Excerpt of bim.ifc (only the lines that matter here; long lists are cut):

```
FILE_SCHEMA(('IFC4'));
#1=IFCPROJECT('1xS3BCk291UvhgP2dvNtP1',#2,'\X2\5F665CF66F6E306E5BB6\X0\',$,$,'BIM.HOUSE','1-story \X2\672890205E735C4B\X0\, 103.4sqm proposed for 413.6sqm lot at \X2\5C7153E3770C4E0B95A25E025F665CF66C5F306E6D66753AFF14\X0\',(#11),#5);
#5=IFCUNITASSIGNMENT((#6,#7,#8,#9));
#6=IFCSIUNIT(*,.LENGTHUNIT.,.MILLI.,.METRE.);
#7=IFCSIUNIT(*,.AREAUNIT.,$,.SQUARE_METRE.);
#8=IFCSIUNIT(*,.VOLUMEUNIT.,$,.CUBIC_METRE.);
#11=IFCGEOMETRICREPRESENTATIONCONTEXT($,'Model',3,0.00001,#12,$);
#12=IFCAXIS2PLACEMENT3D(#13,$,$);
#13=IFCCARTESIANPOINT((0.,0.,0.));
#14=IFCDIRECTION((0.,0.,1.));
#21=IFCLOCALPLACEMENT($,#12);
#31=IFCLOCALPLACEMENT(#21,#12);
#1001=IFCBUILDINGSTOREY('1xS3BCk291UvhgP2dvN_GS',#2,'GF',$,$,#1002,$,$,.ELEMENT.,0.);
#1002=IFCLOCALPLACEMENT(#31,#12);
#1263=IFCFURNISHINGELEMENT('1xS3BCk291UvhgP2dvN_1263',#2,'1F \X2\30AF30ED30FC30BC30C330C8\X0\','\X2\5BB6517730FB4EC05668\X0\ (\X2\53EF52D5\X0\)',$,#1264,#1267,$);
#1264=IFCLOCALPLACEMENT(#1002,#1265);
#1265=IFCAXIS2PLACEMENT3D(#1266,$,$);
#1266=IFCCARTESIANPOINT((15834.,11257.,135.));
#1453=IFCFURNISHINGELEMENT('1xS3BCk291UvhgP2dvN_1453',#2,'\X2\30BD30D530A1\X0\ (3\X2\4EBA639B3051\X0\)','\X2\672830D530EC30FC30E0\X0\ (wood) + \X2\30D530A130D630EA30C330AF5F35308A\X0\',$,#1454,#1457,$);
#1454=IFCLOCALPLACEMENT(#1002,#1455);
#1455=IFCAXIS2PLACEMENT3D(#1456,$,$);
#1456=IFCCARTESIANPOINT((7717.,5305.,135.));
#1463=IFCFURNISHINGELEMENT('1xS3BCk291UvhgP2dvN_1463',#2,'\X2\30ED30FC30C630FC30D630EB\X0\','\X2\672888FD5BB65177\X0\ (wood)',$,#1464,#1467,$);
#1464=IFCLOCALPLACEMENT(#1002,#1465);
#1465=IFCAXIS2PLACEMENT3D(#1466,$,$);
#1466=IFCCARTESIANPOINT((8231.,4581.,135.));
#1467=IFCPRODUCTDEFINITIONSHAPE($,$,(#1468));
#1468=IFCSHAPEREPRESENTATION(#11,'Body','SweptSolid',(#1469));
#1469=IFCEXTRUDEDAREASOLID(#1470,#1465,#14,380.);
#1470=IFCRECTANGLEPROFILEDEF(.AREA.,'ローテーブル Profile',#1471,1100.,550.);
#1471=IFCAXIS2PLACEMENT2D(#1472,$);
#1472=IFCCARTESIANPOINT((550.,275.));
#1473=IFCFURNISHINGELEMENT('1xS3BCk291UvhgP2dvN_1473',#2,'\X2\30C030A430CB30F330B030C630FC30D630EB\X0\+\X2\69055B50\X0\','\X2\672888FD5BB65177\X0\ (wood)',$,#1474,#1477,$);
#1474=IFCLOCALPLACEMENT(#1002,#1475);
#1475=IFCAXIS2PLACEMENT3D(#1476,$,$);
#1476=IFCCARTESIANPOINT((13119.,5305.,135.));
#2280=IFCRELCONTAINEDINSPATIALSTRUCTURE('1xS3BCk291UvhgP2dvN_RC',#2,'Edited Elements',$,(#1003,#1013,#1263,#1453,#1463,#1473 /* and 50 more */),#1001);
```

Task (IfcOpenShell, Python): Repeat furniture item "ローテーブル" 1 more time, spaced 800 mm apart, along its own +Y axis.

```python
import ifcopenshell
import ifcopenshell.api.geometry
import ifcopenshell.api.root
import ifcopenshell.util.element
import ifcopenshell.util.placement
import ifcopenshell.util.unit

model = ifcopenshell.open("bim.ifc")
unit_scale = ifcopenshell.util.unit.calculate_unit_scale(model)


def reuse_history(source, copy):
    """copy_class also copies each property set's owner history, people and application; keep the originals."""
    for rel in copy.IsDefinedBy:
        if rel.is_a("IfcRelDefinesByProperties") and (history := rel.RelatingPropertyDefinition.OwnerHistory):
            rel.RelatingPropertyDefinition.OwnerHistory = source.OwnerHistory
            ifcopenshell.util.element.remove_deep2(model, history)


source = model.by_guid("1xS3BCk291UvhgP2dvN_1463")
base = ifcopenshell.util.placement.get_local_placement(source.ObjectPlacement)
step = base[:3, 1] * 0.8 / unit_scale

for i in range(1, 2):
    copy = ifcopenshell.api.root.copy_class(model, product=source)
    copy.Representation = ifcopenshell.util.element.copy_deep(
        model, source.Representation, exclude=["IfcGeometricRepresentationContext", "IfcRepresentationMap"]
    )
    reuse_history(source, copy)
    matrix = base.copy()
    matrix[:3, 3] += i * step
    print("added at", matrix[:3, 3].round(3) + 0.0)
    ifcopenshell.api.geometry.edit_object_placement(model, product=copy, matrix=matrix, is_si=False)

model.write("bim_edited.ifc")
```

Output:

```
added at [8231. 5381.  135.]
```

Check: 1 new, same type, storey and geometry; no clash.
